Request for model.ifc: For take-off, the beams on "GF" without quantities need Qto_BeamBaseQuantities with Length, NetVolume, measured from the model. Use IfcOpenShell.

First a look at what the model holds.

```python
import ifcopenshell
import ifcopenshell.util.element
import ifcopenshell.util.unit

model = ifcopenshell.open("model.ifc")
print(model.schema)
for unit_type in ("LENGTHUNIT", "AREAUNIT", "VOLUMEUNIT"):
    print(unit_type, ifcopenshell.util.unit.calculate_unit_scale(model, unit_type))
storey = next(s for s in model.by_type("IfcBuildingStorey") if s.Name == "GF")
beams = [e for e in ifcopenshell.util.element.get_decomposition(storey) if e.is_a("IfcBeam")]
for e in sorted(beams, key=lambda e: e.id()):
    print(e.id(), e.is_a(), e.Name, list(ifcopenshell.util.element.get_psets(e, qtos_only=True)), sep=" | ")
```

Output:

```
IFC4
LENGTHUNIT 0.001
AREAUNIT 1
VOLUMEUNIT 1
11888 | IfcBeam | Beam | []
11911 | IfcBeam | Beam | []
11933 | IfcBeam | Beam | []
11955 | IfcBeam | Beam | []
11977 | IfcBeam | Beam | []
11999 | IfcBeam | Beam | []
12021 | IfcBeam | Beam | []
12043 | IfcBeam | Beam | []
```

```python
import ifcopenshell
import ifcopenshell.api.pset
import ifcopenshell.geom
import ifcopenshell.util.element
import ifcopenshell.util.shape
import ifcopenshell.util.unit

model = ifcopenshell.open("model.ifc")
unit_scale = ifcopenshell.util.unit.calculate_unit_scale(model)
volume_scale = ifcopenshell.util.unit.calculate_unit_scale(model, "VOLUMEUNIT")
settings = ifcopenshell.geom.settings()

storey = next(s for s in model.by_type("IfcBuildingStorey") if s.Name == "GF")
beams = [e for e in ifcopenshell.util.element.get_decomposition(storey) if e.is_a("IfcBeam")]

for e in sorted(beams, key=lambda e: e.id()):
    if ifcopenshell.util.element.get_psets(e, qtos_only=True, should_inherit=False):
        continue
    # Geometry comes back in metres, in the element's own axes.
    shape = ifcopenshell.geom.create_shape(settings, e)
    values = {
        "Length": ifcopenshell.util.shape.get_max_xyz(shape.geometry) / unit_scale,
        "NetVolume": ifcopenshell.util.shape.get_volume(shape.geometry) / volume_scale,
    }
    qto = ifcopenshell.api.pset.add_qto(model, product=e, name="Qto_BeamBaseQuantities")
    ifcopenshell.api.pset.edit_qto(model, qto=qto, properties=values)
    print(e.id(), {k: round(v, 3) for k, v in values.items()})

model.write("model_edited.ifc")
```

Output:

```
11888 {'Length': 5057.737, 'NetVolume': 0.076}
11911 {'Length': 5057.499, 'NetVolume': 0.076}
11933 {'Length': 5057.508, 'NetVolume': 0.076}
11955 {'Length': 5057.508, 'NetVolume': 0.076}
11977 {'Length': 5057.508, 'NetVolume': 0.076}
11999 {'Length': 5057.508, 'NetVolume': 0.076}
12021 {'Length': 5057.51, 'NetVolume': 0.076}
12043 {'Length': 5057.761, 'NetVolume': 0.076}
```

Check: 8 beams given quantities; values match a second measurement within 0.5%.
